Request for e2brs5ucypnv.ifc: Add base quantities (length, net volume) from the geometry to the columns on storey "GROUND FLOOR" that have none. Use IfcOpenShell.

First a look at what the model holds.

```python
import ifcopenshell
import ifcopenshell.util.element
import ifcopenshell.util.unit

model = ifcopenshell.open("e2brs5ucypnv.ifc")
print(model.schema)
for unit_type in ("LENGTHUNIT", "AREAUNIT", "VOLUMEUNIT"):
    print(unit_type, ifcopenshell.util.unit.calculate_unit_scale(model, unit_type))
storey = next(s for s in model.by_type("IfcBuildingStorey") if s.Name == "GROUND FLOOR")
columns = [e for e in ifcopenshell.util.element.get_decomposition(storey) if e.is_a("IfcColumn")]
for e in sorted(columns, key=lambda e: e.id()):
    print(e.id(), e.is_a(), e.Name, list(ifcopenshell.util.element.get_psets(e, qtos_only=True)), sep=" | ")
```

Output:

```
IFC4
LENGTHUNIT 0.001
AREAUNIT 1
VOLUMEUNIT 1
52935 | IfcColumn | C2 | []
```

```python
import ifcopenshell
import ifcopenshell.api.pset
import ifcopenshell.geom
import ifcopenshell.util.element
import ifcopenshell.util.shape
import ifcopenshell.util.unit

model = ifcopenshell.open("e2brs5ucypnv.ifc")
unit_scale = ifcopenshell.util.unit.calculate_unit_scale(model)
volume_scale = ifcopenshell.util.unit.calculate_unit_scale(model, "VOLUMEUNIT")
settings = ifcopenshell.geom.settings()

storey = next(s for s in model.by_type("IfcBuildingStorey") if s.Name == "GROUND FLOOR")
columns = [e for e in ifcopenshell.util.element.get_decomposition(storey) if e.is_a("IfcColumn")]

for e in sorted(columns, key=lambda e: e.id()):
    if ifcopenshell.util.element.get_psets(e, qtos_only=True, should_inherit=False):
        continue
    # Geometry comes back in metres, in the element's own axes.
    shape = ifcopenshell.geom.create_shape(settings, e)
    values = {
        "Length": ifcopenshell.util.shape.get_z(shape.geometry) / unit_scale,
        "NetVolume": ifcopenshell.util.shape.get_volume(shape.geometry) / volume_scale,
    }
    qto = ifcopenshell.api.pset.add_qto(model, product=e, name="Qto_ColumnBaseQuantities")
    ifcopenshell.api.pset.edit_qto(model, qto=qto, properties=values)
    print(e.id(), {k: round(v, 3) for k, v in values.items()})

model.write("e2brs5ucypnv_rev.ifc")
```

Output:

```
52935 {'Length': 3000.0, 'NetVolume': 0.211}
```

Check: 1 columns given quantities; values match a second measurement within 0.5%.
